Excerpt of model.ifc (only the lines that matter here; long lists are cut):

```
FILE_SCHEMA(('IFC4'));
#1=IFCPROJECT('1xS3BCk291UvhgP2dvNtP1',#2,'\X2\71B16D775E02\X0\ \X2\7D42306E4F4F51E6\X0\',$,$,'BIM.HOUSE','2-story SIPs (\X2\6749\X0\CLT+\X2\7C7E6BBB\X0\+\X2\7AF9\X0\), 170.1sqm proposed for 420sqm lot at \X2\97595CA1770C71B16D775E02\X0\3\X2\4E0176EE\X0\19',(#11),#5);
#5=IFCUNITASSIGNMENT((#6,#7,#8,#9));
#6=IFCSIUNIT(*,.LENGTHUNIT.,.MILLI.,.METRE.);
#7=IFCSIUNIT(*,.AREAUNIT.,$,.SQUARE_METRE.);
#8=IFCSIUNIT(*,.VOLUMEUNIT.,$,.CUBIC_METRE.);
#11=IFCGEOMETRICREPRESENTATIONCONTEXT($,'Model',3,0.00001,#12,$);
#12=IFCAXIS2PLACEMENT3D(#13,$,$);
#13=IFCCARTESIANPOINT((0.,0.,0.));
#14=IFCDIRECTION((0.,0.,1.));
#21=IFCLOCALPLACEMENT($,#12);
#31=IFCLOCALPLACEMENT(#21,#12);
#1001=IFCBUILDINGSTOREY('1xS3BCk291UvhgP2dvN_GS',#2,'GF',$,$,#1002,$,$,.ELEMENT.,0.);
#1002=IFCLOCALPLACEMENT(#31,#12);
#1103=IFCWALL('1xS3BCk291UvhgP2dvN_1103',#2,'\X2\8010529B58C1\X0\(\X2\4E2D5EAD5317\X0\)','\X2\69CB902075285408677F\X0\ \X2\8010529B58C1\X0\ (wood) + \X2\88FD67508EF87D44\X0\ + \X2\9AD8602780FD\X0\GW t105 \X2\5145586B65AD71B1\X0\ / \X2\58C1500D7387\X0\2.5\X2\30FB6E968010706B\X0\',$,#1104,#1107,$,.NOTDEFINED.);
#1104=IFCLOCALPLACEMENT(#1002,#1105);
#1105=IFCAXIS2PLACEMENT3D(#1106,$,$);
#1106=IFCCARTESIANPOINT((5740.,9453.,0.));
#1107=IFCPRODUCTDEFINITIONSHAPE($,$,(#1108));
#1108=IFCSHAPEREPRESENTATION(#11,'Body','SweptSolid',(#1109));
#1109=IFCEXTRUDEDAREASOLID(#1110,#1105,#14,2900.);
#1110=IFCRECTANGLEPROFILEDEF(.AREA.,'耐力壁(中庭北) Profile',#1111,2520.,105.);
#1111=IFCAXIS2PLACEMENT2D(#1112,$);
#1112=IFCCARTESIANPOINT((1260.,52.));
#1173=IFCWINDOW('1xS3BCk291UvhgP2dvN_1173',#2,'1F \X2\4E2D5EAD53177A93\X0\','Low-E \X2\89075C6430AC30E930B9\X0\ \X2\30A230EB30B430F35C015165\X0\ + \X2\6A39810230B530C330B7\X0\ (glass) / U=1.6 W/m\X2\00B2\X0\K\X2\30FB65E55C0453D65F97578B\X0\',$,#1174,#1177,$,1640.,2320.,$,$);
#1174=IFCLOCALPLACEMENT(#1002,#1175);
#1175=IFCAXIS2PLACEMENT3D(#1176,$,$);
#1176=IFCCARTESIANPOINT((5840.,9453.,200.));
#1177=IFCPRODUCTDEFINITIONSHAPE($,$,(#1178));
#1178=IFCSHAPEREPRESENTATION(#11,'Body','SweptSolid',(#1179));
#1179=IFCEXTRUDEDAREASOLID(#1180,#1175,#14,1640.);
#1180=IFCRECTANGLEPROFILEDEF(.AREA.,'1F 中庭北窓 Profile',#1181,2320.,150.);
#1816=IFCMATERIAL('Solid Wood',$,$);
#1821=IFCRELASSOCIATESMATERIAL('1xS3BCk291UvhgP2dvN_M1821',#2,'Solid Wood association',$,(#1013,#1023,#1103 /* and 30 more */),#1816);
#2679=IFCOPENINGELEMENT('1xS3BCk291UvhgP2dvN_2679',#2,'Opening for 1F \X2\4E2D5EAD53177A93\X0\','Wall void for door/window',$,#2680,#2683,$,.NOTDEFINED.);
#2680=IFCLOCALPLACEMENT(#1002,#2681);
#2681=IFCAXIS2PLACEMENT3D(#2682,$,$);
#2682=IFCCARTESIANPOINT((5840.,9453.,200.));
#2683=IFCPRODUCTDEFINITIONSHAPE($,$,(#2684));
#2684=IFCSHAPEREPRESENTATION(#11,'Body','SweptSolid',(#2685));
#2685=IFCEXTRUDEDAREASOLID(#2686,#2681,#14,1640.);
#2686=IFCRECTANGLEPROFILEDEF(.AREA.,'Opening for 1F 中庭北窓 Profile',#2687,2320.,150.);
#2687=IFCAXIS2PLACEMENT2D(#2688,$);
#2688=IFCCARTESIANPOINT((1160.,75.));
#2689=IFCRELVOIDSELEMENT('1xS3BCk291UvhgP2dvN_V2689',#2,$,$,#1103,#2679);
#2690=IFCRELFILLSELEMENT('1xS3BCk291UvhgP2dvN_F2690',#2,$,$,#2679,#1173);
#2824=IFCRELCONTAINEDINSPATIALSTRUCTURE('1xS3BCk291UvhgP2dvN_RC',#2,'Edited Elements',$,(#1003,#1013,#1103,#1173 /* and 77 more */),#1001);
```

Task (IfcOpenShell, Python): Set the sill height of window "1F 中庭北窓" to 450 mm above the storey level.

```python
import numpy as np
import ifcopenshell
import ifcopenshell.api.geometry
import ifcopenshell.geom
import ifcopenshell.util.element
import ifcopenshell.util.placement
import ifcopenshell.util.shape
import ifcopenshell.util.unit

model = ifcopenshell.open("model.ifc")
unit_scale = ifcopenshell.util.unit.calculate_unit_scale(model)

window = model.by_id(1173)
opening = window.FillsVoids[0].RelatingOpeningElement
storey = ifcopenshell.util.element.get_container(window, ifc_class="IfcBuildingStorey")
level = ifcopenshell.util.placement.get_local_placement(storey.ObjectPlacement)[2, 3]

# The opening's origin need not be at the sill, so measure its lowest point.
shape = ifcopenshell.geom.create_shape(ifcopenshell.geom.settings(), opening)
bottom = ifcopenshell.util.shape.get_shape_bottom_elevation(shape, shape.geometry) / unit_scale
dz = level + 450.0 - bottom

shift = np.array([0.0, 0.0, dz])
# The window is not placed relative to its opening, so move both.
for product in (opening, window):
    matrix = ifcopenshell.util.placement.get_local_placement(product.ObjectPlacement)
    matrix[:3, 3] += shift
    ifcopenshell.api.geometry.edit_object_placement(model, product=product, matrix=matrix, is_si=False)

print(f"moved by {dz * unit_scale:+.3f} m")

model.write("model_v2.ifc")
```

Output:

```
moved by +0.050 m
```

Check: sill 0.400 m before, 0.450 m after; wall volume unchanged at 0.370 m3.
